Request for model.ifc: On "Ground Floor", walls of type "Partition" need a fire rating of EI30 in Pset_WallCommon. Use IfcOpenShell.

First a look at what the model holds.

```python
import ifcopenshell
import ifcopenshell.util.element

model = ifcopenshell.open("model.ifc")
print(model.schema)
storey = next(s for s in model.by_type("IfcBuildingStorey") if s.Name == "Ground Floor")
walls = [e for e in ifcopenshell.util.element.get_decomposition(storey) if e.is_a("IfcWall")]
seen = {}
for e in walls:
    element_type = ifcopenshell.util.element.get_type(e)
    key = (element_type.Name if element_type != e and element_type else None, ifcopenshell.util.element.get_pset(e, "Pset_WallCommon", "FireRating"))
    seen[key] = seen.get(key, 0) + 1
for (name, value), count in sorted(seen.items(), key=str):
    print(count, "x", name, "|", value)
```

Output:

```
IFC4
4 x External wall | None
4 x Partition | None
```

```python
import ifcopenshell
import ifcopenshell.api.pset
import ifcopenshell.util.element

model = ifcopenshell.open("model.ifc")

storey = next(s for s in model.by_type("IfcBuildingStorey") if s.Name == "Ground Floor")
walls = [e for e in ifcopenshell.util.element.get_decomposition(storey) if e.is_a("IfcWall")]

count = 0
for e in walls:
    element_type = ifcopenshell.util.element.get_type(e)
    if element_type in (None, e) or element_type.Name != "Partition":
        continue
    # add_pset returns the element's existing set when there is one.
    pset = ifcopenshell.api.pset.add_pset(model, product=e, name="Pset_WallCommon")
    ifcopenshell.api.pset.edit_pset(model, pset=pset, properties={"FireRating": "EI30"})
    count += 1

print(count, "walls updated")

model.write("model_edited.ifc")
```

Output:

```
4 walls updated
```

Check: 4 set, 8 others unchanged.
